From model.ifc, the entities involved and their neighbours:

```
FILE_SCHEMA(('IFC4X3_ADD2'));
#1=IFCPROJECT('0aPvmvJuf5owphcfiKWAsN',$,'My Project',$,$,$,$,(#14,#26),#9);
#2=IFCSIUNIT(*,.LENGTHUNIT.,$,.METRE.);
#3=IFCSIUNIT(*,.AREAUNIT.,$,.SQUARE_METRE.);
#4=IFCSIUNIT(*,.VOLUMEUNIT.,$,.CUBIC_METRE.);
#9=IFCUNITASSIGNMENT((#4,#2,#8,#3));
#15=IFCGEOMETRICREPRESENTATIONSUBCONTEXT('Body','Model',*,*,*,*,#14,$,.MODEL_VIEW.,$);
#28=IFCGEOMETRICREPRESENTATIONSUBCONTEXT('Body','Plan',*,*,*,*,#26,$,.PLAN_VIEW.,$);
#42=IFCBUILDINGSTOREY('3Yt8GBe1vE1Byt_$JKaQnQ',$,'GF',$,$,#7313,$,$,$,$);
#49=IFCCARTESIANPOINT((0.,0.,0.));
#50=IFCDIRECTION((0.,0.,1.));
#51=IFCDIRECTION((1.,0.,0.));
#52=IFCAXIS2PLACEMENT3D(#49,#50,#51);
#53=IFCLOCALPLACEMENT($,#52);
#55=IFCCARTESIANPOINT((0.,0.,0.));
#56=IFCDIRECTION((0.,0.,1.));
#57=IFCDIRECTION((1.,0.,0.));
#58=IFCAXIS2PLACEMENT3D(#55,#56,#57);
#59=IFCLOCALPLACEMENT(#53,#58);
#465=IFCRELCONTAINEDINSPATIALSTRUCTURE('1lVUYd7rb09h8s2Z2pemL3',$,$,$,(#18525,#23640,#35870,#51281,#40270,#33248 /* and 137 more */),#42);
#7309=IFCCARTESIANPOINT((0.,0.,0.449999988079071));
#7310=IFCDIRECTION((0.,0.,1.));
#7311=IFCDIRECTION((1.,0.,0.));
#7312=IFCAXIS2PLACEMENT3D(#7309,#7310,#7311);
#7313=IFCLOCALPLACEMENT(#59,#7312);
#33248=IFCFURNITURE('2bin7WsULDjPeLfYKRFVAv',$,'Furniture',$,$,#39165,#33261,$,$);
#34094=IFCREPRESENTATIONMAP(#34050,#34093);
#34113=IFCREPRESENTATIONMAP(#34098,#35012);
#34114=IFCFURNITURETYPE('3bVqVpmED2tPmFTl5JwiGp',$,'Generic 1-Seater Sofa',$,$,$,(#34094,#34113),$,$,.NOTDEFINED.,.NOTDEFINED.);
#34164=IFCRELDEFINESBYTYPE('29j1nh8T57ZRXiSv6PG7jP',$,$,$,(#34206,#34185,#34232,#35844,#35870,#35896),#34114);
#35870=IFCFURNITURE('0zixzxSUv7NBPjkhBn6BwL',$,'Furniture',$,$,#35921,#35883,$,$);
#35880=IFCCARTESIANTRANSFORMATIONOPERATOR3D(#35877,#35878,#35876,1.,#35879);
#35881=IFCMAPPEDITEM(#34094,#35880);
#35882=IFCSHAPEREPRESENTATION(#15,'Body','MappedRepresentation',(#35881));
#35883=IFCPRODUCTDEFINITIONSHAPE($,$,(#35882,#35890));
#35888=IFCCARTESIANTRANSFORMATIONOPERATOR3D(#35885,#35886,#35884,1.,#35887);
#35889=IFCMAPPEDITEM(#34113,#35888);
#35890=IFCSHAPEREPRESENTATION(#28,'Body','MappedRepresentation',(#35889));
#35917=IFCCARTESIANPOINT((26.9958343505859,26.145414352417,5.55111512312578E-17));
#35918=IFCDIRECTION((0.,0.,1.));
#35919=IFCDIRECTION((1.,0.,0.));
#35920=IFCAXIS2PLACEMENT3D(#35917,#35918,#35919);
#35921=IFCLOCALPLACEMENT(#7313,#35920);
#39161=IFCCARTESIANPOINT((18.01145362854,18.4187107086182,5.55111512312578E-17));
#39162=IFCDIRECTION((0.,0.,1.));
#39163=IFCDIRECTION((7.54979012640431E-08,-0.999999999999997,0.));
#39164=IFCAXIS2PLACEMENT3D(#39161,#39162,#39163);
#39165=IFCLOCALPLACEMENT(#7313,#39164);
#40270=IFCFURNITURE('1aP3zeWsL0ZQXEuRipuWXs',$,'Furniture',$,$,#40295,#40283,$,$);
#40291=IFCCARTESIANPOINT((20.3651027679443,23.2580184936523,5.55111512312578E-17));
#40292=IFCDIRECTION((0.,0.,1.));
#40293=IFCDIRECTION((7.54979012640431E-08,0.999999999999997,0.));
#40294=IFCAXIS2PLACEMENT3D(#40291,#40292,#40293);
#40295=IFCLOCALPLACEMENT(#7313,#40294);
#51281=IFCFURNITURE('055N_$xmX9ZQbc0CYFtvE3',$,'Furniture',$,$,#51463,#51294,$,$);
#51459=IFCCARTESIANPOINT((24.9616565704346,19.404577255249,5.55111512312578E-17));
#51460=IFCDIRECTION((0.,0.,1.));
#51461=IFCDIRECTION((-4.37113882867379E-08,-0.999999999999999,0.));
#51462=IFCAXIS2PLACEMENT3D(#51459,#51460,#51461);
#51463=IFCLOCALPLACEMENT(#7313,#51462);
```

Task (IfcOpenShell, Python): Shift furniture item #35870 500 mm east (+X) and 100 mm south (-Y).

```python
import ifcopenshell
import ifcopenshell.api.geometry
import ifcopenshell.util.placement

model = ifcopenshell.open("model.ifc")

item = model.by_guid("0zixzxSUv7NBPjkhBn6BwL")
matrix = ifcopenshell.util.placement.get_local_placement(item.ObjectPlacement)
matrix[0, 3] += 0.5
matrix[1, 3] -= 0.1
ifcopenshell.api.geometry.edit_object_placement(model, product=item, matrix=matrix, is_si=False)

print(ifcopenshell.util.placement.get_local_placement(item.ObjectPlacement).round(3) + 0.0)

model.write("model_edited.ifc")
```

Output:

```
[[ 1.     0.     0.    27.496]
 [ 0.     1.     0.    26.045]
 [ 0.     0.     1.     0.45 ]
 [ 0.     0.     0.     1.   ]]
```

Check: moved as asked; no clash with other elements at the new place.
